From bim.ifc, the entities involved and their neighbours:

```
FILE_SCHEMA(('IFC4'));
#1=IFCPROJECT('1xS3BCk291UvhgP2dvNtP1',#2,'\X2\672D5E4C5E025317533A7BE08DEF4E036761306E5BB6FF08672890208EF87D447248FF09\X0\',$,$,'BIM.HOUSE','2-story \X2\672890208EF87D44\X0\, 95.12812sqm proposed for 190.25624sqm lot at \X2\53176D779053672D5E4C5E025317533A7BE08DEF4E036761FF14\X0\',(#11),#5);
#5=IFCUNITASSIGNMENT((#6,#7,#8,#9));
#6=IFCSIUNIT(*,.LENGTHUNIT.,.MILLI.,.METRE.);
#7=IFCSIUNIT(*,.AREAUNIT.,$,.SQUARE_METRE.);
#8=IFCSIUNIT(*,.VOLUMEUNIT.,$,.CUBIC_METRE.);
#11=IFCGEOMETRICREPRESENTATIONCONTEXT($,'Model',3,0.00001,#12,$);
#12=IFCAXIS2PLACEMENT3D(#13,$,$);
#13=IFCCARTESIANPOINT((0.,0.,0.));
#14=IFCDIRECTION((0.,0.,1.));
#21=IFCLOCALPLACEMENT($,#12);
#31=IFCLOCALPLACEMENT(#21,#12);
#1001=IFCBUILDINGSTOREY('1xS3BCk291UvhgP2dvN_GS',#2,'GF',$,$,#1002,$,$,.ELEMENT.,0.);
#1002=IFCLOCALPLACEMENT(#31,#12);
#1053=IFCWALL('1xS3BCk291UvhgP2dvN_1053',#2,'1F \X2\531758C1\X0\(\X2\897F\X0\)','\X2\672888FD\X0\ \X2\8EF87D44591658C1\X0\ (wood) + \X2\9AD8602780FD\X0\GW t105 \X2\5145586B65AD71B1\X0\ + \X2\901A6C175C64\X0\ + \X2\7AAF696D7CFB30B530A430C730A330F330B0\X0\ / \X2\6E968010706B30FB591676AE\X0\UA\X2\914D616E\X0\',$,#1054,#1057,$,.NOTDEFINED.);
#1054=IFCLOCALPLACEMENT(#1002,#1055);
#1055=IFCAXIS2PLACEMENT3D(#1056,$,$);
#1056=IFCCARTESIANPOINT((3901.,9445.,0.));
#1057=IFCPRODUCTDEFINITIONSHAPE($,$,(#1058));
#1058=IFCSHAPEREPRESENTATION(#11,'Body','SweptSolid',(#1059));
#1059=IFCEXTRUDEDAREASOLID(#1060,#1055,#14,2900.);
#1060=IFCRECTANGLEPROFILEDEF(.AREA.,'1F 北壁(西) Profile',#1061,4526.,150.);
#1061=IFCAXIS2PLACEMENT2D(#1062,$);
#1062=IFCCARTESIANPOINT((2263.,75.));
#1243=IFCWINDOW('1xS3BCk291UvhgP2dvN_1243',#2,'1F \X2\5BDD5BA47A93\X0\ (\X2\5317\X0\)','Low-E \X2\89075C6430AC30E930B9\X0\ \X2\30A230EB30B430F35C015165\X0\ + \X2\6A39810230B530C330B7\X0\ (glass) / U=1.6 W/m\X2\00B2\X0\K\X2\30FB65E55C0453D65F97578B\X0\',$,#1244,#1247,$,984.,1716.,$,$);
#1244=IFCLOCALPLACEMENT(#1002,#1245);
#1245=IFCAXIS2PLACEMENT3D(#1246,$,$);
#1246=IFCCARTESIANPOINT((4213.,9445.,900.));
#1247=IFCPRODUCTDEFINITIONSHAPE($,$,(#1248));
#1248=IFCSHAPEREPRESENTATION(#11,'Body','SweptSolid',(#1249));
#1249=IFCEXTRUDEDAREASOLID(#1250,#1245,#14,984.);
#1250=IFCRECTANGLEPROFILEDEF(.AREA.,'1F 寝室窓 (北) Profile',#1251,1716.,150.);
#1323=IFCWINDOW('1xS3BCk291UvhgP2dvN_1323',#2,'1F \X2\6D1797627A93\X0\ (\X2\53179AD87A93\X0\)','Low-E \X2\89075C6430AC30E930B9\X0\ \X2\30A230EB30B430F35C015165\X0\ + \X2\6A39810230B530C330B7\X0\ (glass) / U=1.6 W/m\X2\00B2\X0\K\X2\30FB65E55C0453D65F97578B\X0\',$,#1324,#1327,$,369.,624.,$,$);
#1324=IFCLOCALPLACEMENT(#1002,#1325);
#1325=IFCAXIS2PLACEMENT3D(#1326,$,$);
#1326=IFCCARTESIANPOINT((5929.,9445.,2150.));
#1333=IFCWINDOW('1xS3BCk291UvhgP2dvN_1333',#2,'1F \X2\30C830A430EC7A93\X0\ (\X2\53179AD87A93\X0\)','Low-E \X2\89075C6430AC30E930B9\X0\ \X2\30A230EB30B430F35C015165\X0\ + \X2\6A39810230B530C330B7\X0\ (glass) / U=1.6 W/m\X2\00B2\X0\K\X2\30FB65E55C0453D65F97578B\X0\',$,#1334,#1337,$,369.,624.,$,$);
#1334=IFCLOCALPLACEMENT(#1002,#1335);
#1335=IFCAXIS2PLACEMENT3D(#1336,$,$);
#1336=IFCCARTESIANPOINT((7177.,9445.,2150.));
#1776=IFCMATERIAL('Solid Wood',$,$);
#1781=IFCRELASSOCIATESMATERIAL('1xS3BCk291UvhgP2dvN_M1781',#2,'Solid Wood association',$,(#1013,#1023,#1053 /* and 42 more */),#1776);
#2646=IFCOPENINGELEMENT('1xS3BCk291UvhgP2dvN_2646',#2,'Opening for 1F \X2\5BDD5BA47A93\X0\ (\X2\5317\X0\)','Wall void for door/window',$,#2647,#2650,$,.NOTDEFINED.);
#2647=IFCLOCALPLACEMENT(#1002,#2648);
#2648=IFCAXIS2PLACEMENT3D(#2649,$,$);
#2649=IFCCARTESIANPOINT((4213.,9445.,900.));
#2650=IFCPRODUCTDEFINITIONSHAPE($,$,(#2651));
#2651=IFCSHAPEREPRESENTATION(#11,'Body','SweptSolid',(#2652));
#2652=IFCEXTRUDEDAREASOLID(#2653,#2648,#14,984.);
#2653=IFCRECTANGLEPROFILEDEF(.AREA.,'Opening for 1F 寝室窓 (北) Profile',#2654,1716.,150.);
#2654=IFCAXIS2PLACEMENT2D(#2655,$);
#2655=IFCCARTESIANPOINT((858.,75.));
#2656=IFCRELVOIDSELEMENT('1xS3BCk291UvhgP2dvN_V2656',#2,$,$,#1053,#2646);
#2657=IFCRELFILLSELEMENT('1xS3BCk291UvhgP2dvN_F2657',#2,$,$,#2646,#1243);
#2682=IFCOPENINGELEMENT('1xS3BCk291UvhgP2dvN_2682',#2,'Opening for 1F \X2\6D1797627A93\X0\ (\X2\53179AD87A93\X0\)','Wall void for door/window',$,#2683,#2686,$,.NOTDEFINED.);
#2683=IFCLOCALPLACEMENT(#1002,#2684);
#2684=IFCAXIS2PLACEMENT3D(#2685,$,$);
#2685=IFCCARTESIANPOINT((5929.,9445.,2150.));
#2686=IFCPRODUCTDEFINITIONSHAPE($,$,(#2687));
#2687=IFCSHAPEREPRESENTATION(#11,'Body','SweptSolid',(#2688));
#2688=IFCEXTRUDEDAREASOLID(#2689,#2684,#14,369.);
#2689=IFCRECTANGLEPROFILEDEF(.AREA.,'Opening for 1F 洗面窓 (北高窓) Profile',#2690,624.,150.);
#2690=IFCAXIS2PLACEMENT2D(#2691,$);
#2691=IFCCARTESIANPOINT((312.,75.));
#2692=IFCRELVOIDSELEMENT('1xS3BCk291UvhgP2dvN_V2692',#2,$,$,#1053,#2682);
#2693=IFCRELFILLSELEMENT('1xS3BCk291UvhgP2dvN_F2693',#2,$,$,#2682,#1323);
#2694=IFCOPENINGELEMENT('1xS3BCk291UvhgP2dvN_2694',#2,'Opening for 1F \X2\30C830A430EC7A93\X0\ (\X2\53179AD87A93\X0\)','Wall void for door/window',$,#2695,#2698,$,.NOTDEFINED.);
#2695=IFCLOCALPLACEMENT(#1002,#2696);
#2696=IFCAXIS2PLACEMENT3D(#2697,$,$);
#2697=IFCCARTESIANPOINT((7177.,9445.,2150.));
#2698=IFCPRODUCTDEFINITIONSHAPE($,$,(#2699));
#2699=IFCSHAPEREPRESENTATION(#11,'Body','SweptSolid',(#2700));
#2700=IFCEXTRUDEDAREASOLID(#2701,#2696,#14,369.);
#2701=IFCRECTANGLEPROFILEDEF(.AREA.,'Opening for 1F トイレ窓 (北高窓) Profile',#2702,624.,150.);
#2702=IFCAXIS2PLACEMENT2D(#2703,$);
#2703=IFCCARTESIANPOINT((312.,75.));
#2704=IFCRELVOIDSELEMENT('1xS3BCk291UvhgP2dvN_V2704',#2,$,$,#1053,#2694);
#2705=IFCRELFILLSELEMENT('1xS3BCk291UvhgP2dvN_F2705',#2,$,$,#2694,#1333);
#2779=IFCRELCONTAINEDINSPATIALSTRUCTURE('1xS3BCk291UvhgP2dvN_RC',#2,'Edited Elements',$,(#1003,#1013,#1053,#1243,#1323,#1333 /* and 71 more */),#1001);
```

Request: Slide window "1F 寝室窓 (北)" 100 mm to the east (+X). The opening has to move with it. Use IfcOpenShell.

```python
import ifcopenshell
import ifcopenshell.api.geometry
import ifcopenshell.util.placement

model = ifcopenshell.open("bim.ifc")

window = model.by_guid("1xS3BCk291UvhgP2dvN_1243")
opening = window.FillsVoids[0].RelatingOpeningElement
wall = opening.VoidsElements[0].RelatingBuildingElement

wall_matrix = ifcopenshell.util.placement.get_local_placement(wall.ObjectPlacement)
shift = wall_matrix[:3, 0] * 100.0
before = ifcopenshell.util.placement.get_local_placement(window.ObjectPlacement)[:3, 3].copy()

# The window is not placed relative to its opening, so move both.
for product in (opening, window):
    matrix = ifcopenshell.util.placement.get_local_placement(product.ObjectPlacement)
    matrix[:3, 3] += shift
    ifcopenshell.api.geometry.edit_object_placement(model, product=product, matrix=matrix, is_si=False)

after = ifcopenshell.util.placement.get_local_placement(window.ObjectPlacement)[:3, 3]
print("window moved by", (after - before).round(3) + 0.0)

model.write("bim_rev.ifc")
```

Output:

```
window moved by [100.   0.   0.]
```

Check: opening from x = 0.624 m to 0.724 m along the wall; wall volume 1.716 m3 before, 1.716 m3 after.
